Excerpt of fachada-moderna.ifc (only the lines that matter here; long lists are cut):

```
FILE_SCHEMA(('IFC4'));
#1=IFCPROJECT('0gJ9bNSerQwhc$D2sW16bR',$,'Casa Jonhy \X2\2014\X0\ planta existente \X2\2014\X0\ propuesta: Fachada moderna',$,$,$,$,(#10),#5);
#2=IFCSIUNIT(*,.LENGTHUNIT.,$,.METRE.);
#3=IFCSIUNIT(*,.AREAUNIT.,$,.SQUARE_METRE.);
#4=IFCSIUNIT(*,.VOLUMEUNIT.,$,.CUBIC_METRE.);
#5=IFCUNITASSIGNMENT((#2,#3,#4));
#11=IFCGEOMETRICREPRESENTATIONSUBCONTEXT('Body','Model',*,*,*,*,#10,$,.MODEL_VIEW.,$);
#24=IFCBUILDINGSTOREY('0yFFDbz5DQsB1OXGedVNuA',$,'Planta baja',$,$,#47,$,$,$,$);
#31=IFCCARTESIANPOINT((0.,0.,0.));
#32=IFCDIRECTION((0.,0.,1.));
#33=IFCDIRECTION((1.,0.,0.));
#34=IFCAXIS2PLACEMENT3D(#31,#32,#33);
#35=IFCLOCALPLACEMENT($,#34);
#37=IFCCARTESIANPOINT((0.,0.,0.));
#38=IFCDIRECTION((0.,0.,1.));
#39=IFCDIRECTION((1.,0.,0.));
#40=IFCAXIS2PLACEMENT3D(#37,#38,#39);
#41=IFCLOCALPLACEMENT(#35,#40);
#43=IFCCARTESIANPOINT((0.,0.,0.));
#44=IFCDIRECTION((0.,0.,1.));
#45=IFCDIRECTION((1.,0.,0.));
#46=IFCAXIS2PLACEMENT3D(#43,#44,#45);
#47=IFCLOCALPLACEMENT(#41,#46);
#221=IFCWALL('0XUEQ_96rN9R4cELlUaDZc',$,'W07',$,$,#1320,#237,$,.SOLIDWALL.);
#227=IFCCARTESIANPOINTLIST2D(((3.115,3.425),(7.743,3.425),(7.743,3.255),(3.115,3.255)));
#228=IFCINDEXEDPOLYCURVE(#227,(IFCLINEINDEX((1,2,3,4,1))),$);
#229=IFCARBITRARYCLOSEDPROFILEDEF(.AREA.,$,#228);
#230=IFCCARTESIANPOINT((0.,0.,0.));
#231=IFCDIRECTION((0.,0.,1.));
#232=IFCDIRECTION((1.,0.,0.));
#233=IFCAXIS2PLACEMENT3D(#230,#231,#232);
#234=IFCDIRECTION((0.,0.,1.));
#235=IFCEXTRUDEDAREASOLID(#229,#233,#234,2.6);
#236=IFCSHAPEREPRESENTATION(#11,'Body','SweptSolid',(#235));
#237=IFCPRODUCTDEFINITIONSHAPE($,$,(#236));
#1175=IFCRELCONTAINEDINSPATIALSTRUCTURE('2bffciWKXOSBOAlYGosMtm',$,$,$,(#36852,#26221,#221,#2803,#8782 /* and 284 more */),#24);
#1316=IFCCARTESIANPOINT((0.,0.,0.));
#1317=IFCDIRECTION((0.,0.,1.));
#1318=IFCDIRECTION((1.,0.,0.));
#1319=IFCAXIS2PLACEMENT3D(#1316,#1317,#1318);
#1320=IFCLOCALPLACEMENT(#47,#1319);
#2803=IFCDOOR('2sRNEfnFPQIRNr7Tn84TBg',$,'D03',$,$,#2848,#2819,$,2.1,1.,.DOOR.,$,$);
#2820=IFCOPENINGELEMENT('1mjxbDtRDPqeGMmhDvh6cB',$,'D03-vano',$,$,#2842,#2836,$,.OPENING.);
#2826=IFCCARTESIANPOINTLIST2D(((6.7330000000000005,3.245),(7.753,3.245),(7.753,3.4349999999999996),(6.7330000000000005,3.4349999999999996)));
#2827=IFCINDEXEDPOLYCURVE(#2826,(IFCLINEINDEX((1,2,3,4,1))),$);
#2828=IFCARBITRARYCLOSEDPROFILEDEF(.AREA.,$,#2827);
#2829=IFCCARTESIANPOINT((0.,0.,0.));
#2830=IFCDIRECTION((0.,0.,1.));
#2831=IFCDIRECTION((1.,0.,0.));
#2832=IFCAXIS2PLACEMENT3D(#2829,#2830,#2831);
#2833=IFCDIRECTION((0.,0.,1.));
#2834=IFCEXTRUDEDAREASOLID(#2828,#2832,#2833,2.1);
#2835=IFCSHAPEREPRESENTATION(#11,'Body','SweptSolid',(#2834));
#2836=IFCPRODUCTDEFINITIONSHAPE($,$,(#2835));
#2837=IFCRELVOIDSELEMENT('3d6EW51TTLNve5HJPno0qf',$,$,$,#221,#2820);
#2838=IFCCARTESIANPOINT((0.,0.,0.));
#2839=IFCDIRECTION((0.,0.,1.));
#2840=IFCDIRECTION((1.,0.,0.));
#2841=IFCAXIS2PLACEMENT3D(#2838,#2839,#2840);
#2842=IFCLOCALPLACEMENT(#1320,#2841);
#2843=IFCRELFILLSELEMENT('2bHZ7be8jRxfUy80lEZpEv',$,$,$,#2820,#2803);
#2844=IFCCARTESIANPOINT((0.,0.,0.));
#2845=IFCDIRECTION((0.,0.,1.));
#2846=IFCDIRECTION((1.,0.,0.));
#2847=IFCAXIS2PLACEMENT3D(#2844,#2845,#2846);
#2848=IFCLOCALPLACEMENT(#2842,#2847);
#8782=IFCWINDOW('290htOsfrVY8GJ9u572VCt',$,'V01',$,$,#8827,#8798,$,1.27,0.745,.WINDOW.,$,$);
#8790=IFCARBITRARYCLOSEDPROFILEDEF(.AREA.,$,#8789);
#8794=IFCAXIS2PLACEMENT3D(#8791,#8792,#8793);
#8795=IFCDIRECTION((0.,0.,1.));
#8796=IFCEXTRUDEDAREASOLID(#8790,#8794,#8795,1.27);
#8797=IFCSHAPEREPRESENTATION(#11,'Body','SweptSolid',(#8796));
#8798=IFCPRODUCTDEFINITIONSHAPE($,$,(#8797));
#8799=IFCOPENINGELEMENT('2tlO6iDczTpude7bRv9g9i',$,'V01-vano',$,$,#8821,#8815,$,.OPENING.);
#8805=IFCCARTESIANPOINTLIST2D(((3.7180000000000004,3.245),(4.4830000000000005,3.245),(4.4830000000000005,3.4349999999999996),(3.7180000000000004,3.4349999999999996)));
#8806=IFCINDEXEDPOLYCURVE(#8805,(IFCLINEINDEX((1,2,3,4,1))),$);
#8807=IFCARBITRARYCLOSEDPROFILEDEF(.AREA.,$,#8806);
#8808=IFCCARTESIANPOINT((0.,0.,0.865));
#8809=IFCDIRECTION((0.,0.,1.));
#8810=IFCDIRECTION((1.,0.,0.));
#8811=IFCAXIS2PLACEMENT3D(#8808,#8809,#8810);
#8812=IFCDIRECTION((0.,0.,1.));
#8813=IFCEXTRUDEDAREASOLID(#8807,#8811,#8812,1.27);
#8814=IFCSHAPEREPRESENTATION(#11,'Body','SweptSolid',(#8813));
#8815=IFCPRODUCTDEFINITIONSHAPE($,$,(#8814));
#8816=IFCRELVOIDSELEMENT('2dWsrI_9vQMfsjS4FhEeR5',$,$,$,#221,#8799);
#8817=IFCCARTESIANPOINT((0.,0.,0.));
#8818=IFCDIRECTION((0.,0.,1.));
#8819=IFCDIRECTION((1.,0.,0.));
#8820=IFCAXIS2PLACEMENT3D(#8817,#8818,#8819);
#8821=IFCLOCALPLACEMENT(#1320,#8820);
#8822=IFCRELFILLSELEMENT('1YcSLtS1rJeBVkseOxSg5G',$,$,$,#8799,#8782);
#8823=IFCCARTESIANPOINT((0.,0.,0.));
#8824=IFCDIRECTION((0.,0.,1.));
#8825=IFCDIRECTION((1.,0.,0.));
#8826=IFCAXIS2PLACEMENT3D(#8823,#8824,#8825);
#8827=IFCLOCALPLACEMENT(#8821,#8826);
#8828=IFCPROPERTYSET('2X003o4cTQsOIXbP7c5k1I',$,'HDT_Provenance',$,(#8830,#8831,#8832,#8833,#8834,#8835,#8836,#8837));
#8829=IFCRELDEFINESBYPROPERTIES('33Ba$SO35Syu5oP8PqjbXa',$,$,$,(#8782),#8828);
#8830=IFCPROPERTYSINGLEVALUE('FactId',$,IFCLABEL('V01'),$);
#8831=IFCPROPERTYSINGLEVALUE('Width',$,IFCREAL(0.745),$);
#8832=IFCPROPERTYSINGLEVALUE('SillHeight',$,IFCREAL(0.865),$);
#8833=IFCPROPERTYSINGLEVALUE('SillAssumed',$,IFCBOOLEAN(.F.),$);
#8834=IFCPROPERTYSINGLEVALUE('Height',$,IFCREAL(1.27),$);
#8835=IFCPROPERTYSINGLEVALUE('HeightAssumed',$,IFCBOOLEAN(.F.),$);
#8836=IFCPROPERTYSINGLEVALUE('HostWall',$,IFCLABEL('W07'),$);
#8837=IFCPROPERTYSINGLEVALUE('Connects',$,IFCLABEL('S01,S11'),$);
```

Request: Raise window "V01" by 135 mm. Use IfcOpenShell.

```python
import numpy as np
import ifcopenshell
import ifcopenshell.api.geometry
import ifcopenshell.api.pset
import ifcopenshell.util.element
import ifcopenshell.util.placement
import ifcopenshell.util.unit

model = ifcopenshell.open("fachada-moderna.ifc")
unit_scale = ifcopenshell.util.unit.calculate_unit_scale(model)

window = model.by_id(8782)
opening = window.FillsVoids[0].RelatingOpeningElement
dz = 0.135 / unit_scale

shift = np.array([0.0, 0.0, dz])
# The window is placed relative to its opening, so it follows when the opening moves.
matrix = ifcopenshell.util.placement.get_local_placement(opening.ObjectPlacement)
matrix[:3, 3] += shift
ifcopenshell.api.geometry.edit_object_placement(
    model, product=opening, matrix=matrix, is_si=False, should_transform_children=True
)

# Keep the stored heights in step.
pset = model.by_id(ifcopenshell.util.element.get_pset(window, "HDT_Provenance", should_inherit=False)["id"])
ifcopenshell.api.pset.edit_pset(model, pset=pset, properties={
    "SillHeight": model.create_entity("IfcReal", ifcopenshell.util.element.get_pset(window, "HDT_Provenance", "SillHeight") + dz),
})

print(f"moved by {dz * unit_scale:+.3f} m")

model.write("fachada-moderna_rev.ifc")
```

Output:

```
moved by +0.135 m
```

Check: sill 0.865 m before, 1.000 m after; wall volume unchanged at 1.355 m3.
